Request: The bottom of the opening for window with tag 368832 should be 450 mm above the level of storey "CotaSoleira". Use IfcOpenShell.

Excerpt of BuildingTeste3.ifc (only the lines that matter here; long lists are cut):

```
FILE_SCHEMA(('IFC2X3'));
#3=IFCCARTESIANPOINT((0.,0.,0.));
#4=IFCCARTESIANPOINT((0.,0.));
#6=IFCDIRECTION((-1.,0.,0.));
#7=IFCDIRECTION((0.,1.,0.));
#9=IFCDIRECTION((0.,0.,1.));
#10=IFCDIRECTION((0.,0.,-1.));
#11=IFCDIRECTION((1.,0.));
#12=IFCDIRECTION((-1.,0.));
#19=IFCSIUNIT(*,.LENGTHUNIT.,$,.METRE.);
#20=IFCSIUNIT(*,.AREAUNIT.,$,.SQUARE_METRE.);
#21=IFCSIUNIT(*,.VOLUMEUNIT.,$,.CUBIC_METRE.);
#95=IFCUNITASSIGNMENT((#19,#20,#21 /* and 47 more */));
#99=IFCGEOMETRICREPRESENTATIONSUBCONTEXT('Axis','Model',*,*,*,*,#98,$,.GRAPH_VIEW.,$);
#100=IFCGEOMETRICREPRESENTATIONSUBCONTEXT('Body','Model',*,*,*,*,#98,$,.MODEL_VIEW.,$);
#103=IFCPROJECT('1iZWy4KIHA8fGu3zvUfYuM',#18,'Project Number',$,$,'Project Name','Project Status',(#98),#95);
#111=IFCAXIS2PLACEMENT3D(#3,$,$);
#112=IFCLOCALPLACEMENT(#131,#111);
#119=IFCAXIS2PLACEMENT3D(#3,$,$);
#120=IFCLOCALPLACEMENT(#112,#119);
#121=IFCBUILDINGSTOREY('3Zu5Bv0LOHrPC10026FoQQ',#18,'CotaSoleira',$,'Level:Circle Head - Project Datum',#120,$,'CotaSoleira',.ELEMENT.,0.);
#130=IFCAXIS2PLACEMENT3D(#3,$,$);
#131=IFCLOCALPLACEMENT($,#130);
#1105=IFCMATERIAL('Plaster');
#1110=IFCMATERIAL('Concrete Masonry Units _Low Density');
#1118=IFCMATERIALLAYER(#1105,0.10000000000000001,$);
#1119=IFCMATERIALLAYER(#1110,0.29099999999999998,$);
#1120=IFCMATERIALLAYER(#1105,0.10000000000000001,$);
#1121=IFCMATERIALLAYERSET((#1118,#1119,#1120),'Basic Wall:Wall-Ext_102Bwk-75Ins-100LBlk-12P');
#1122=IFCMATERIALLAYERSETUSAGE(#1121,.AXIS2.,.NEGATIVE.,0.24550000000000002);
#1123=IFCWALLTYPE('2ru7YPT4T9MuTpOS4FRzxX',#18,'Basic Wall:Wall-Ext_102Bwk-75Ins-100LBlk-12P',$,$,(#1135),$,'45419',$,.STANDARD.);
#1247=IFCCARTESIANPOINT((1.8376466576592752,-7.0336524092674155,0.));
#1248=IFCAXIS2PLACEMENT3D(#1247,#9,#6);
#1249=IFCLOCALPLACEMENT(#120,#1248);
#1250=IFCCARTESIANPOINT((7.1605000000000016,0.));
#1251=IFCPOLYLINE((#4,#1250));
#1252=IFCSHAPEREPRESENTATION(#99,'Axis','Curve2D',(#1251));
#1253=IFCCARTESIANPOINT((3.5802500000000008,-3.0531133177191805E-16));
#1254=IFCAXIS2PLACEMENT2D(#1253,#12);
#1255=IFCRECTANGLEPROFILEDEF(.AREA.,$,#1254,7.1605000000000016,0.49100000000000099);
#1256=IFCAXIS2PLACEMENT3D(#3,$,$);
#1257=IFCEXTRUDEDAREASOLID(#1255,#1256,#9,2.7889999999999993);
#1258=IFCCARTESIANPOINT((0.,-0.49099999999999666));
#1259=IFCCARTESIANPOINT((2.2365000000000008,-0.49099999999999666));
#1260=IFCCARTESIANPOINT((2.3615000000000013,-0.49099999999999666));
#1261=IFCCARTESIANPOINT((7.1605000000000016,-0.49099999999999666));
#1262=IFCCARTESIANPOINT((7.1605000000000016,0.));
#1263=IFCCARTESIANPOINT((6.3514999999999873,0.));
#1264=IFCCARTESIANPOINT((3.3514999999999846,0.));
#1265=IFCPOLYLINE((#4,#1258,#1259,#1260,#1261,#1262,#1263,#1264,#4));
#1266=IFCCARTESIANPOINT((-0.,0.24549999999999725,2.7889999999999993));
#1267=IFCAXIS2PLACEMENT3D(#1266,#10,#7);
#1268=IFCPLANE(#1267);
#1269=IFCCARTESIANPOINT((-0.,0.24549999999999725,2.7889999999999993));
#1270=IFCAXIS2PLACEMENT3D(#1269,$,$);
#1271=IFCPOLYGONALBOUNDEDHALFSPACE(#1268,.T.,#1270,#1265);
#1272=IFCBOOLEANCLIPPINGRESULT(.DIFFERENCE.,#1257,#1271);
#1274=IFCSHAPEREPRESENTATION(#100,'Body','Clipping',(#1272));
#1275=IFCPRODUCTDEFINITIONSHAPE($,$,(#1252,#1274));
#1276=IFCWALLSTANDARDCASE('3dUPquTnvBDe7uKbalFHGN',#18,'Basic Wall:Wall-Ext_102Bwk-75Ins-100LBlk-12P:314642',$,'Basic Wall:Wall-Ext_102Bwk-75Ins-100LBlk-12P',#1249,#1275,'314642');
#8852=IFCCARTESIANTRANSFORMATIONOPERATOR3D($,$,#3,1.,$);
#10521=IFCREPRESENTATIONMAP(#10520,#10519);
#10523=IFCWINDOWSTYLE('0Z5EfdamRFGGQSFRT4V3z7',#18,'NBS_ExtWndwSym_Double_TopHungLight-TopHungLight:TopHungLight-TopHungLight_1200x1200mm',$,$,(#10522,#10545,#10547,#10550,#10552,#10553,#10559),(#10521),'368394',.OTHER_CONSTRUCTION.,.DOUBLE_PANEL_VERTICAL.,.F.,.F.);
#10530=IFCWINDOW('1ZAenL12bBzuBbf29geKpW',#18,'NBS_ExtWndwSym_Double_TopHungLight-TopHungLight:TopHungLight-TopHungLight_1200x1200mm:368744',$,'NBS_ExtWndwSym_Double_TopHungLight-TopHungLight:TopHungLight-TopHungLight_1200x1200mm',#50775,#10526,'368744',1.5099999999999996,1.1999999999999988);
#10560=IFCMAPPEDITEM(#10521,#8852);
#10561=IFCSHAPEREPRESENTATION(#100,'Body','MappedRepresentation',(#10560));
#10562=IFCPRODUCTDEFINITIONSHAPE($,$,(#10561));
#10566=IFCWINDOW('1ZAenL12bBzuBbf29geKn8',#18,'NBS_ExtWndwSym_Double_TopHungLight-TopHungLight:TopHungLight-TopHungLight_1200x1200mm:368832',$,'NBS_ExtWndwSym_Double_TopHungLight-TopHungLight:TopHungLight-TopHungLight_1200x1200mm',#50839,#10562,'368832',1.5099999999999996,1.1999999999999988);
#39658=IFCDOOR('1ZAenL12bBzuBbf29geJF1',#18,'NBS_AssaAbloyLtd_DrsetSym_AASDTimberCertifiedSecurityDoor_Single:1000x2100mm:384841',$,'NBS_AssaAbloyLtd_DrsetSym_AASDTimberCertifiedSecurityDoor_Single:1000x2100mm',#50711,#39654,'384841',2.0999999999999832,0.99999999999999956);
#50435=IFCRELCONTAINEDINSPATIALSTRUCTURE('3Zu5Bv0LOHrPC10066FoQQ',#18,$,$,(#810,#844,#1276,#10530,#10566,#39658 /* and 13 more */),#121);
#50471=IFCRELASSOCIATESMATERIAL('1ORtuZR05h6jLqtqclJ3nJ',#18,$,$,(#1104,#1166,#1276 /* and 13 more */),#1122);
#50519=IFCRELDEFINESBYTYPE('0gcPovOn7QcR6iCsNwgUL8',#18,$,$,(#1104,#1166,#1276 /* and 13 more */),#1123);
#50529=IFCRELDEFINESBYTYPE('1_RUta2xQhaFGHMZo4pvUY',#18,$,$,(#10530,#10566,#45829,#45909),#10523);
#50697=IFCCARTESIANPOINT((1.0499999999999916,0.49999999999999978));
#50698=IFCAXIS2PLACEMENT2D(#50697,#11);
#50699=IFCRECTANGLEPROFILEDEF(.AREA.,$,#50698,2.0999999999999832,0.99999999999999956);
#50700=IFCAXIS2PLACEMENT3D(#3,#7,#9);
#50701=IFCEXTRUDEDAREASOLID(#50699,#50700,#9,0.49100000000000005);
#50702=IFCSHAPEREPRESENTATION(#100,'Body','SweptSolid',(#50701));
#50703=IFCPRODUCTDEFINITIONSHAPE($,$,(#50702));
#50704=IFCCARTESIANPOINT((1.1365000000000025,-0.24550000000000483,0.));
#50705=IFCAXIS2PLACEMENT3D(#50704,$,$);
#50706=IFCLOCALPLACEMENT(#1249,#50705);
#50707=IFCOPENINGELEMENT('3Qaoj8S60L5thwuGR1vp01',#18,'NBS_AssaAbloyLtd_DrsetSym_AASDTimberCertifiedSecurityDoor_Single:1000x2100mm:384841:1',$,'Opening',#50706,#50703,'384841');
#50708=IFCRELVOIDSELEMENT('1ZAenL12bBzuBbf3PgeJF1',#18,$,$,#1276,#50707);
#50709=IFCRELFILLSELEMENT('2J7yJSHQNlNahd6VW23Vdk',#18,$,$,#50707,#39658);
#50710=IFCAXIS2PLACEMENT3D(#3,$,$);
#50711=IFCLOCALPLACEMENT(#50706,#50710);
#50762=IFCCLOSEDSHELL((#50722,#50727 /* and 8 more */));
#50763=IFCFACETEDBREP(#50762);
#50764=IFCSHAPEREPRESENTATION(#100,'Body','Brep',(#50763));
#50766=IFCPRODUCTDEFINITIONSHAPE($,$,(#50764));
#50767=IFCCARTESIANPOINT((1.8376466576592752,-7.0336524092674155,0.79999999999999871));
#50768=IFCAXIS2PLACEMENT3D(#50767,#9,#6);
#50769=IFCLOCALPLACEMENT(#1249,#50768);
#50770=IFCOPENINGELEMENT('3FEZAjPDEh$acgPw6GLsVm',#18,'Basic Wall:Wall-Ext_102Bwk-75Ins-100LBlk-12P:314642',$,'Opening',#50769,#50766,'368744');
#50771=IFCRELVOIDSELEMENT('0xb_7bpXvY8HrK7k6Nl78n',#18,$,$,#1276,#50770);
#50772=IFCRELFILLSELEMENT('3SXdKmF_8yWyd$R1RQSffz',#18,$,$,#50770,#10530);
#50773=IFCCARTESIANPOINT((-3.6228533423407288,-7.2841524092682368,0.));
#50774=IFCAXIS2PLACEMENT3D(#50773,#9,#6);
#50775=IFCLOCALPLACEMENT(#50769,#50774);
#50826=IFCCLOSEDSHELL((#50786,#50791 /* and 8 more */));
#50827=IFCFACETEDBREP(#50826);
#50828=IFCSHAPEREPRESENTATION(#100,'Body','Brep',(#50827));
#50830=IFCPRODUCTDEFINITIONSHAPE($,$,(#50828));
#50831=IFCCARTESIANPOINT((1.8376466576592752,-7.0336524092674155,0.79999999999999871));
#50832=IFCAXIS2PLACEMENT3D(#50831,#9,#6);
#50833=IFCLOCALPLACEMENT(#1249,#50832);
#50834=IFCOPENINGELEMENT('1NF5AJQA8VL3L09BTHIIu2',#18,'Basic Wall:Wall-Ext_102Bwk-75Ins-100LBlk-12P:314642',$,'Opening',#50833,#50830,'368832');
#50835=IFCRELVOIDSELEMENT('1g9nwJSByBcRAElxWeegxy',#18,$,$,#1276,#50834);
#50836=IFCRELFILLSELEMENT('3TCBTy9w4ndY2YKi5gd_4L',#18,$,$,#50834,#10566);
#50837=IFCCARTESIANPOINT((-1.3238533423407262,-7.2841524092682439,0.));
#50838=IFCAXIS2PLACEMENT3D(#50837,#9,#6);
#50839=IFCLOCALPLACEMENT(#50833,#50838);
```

```python
import numpy as np
import ifcopenshell
import ifcopenshell.api.geometry
import ifcopenshell.geom
import ifcopenshell.util.element
import ifcopenshell.util.placement
import ifcopenshell.util.shape
import ifcopenshell.util.unit

model = ifcopenshell.open("BuildingTeste3.ifc")
unit_scale = ifcopenshell.util.unit.calculate_unit_scale(model)

window = model.by_guid("1ZAenL12bBzuBbf29geKn8")
opening = window.FillsVoids[0].RelatingOpeningElement
storey = ifcopenshell.util.element.get_container(window, ifc_class="IfcBuildingStorey")
level = ifcopenshell.util.placement.get_local_placement(storey.ObjectPlacement)[2, 3]

# The opening's origin need not be at the sill, so measure its lowest point.
shape = ifcopenshell.geom.create_shape(ifcopenshell.geom.settings(), opening)
bottom = ifcopenshell.util.shape.get_shape_bottom_elevation(shape, shape.geometry) / unit_scale
dz = level + 0.45 - bottom

shift = np.array([0.0, 0.0, dz])
# The window is placed relative to its opening, so it follows when the opening moves.
matrix = ifcopenshell.util.placement.get_local_placement(opening.ObjectPlacement)
matrix[:3, 3] += shift
ifcopenshell.api.geometry.edit_object_placement(
    model, product=opening, matrix=matrix, is_si=False, should_transform_children=True
)

print(f"moved by {dz * unit_scale:+.3f} m")

model.write("BuildingTeste3_edited.ifc")
```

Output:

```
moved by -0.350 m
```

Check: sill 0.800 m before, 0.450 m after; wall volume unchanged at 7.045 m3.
